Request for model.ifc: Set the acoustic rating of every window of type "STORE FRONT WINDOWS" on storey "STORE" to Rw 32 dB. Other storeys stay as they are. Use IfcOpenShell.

First a look at what the model holds.

```python
import ifcopenshell
import ifcopenshell.util.element

model = ifcopenshell.open("model.ifc")
print(model.schema)
storey = next(s for s in model.by_type("IfcBuildingStorey") if s.Name == "STORE")
windows = [e for e in ifcopenshell.util.element.get_decomposition(storey) if e.is_a("IfcWindow")]
seen = {}
for e in windows:
    element_type = ifcopenshell.util.element.get_type(e)
    key = (element_type.Name if element_type != e and element_type else None, ifcopenshell.util.element.get_pset(e, "Pset_WindowCommon", "AcousticRating"))
    seen[key] = seen.get(key, 0) + 1
for (name, value), count in sorted(seen.items(), key=str):
    print(count, "x", name, "|", value)
```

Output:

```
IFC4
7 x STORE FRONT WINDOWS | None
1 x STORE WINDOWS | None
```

```python
import ifcopenshell
import ifcopenshell.api.pset
import ifcopenshell.util.element

model = ifcopenshell.open("model.ifc")

storey = next(s for s in model.by_type("IfcBuildingStorey") if s.Name == "STORE")
windows = [e for e in ifcopenshell.util.element.get_decomposition(storey) if e.is_a("IfcWindow")]

count = 0
for e in windows:
    element_type = ifcopenshell.util.element.get_type(e)
    if element_type in (None, e) or element_type.Name != "STORE FRONT WINDOWS":
        continue
    # add_pset returns the element's existing set when there is one.
    pset = ifcopenshell.api.pset.add_pset(model, product=e, name="Pset_WindowCommon")
    ifcopenshell.api.pset.edit_pset(model, pset=pset, properties={"AcousticRating": "Rw 32 dB"})
    count += 1

print(count, "windows updated")

model.write("model_rev.ifc")
```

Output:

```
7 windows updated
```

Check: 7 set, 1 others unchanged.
